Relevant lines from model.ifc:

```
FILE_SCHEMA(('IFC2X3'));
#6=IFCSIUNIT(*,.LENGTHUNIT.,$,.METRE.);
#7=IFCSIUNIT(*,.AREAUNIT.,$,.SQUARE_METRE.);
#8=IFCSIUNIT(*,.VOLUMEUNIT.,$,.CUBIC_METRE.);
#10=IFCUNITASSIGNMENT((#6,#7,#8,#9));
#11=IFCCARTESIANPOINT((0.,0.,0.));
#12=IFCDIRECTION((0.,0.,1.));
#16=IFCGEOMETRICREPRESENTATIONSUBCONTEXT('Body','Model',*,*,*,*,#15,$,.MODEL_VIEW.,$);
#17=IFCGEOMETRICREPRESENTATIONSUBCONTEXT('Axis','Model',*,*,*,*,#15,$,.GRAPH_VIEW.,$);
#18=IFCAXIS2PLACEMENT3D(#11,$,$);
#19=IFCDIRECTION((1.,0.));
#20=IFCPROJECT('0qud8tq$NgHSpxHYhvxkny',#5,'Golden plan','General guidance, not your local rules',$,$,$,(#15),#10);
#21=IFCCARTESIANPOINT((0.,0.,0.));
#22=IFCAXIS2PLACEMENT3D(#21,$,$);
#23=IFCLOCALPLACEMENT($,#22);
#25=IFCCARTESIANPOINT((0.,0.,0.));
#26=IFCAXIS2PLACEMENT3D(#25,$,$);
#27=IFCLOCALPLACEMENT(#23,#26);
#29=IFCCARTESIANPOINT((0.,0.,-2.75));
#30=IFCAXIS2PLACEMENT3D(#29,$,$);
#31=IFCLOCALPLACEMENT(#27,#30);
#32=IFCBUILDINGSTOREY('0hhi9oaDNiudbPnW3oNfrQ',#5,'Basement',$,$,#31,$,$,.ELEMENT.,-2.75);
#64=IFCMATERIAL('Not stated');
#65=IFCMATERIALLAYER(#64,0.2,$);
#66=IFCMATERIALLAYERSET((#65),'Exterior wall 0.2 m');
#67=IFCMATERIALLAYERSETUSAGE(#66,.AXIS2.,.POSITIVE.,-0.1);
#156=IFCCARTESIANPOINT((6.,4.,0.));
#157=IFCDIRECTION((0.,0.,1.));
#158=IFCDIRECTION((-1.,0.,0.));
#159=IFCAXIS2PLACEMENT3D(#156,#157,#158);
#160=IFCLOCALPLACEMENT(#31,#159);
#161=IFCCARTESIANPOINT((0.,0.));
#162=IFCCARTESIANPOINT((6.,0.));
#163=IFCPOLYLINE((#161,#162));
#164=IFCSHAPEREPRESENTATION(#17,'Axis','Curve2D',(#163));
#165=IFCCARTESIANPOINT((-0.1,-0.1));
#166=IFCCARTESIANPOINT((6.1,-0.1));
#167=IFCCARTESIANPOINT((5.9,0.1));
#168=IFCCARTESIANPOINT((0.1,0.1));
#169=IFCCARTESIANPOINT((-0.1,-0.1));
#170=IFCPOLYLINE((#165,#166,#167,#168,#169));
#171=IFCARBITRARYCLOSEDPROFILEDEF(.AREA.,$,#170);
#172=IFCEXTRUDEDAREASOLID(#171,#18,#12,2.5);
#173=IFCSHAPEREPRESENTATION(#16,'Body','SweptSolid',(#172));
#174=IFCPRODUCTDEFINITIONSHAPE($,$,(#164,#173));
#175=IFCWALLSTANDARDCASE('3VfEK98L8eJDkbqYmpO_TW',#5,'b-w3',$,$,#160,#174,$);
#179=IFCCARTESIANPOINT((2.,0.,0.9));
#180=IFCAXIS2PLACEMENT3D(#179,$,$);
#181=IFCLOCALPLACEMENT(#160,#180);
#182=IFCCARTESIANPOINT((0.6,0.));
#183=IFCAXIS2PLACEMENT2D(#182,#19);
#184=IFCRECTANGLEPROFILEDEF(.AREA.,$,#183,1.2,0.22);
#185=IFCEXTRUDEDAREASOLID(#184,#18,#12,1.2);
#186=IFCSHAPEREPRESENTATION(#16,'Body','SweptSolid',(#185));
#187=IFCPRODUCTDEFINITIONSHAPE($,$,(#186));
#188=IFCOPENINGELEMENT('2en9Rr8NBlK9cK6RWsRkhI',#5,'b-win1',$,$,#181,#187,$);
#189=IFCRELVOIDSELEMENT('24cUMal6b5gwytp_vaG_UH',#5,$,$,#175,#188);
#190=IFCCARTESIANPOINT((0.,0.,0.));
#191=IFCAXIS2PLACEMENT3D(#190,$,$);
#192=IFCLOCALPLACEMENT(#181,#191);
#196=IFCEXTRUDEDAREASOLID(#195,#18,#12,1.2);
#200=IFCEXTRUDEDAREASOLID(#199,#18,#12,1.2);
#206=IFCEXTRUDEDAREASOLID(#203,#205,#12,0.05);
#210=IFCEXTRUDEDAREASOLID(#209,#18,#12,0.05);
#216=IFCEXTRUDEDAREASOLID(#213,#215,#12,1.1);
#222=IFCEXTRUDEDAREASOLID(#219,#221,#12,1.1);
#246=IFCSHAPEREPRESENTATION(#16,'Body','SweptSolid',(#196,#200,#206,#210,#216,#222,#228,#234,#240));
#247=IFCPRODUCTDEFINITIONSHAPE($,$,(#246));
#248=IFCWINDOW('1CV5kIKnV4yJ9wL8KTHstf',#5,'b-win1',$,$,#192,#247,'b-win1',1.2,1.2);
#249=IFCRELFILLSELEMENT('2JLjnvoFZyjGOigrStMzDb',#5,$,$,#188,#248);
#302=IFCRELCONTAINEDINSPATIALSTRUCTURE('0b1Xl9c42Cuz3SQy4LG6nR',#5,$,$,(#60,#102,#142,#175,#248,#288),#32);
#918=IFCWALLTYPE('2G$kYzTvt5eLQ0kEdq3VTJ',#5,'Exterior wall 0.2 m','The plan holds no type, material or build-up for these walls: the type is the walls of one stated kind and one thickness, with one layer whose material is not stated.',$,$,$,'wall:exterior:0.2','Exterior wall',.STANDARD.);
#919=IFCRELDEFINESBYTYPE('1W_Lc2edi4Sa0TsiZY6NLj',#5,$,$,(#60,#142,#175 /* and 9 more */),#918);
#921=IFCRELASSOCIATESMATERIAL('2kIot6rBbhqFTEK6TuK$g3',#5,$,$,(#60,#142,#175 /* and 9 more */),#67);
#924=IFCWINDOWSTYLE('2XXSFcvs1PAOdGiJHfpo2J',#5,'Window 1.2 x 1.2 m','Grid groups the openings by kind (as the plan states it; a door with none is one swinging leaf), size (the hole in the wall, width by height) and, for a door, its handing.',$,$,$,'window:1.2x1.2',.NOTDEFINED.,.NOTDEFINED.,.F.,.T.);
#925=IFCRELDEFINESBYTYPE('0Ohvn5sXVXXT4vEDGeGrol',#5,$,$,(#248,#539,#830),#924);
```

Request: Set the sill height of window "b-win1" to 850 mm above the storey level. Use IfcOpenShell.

```python
import numpy as np
import ifcopenshell
import ifcopenshell.api.geometry
import ifcopenshell.geom
import ifcopenshell.util.element
import ifcopenshell.util.placement
import ifcopenshell.util.shape
import ifcopenshell.util.unit

model = ifcopenshell.open("model.ifc")
unit_scale = ifcopenshell.util.unit.calculate_unit_scale(model)

window = model.by_id(248)
opening = window.FillsVoids[0].RelatingOpeningElement
storey = ifcopenshell.util.element.get_container(window, ifc_class="IfcBuildingStorey")
level = ifcopenshell.util.placement.get_local_placement(storey.ObjectPlacement)[2, 3]

# The opening's origin need not be at the sill, so measure its lowest point.
shape = ifcopenshell.geom.create_shape(ifcopenshell.geom.settings(), opening)
bottom = ifcopenshell.util.shape.get_shape_bottom_elevation(shape, shape.geometry) / unit_scale
dz = level + 0.85 - bottom

shift = np.array([0.0, 0.0, dz])
# The window is placed relative to its opening, so it follows when the opening moves.
matrix = ifcopenshell.util.placement.get_local_placement(opening.ObjectPlacement)
matrix[:3, 3] += shift
ifcopenshell.api.geometry.edit_object_placement(
    model, product=opening, matrix=matrix, is_si=False, should_transform_children=True
)

print(f"moved by {dz * unit_scale:+.3f} m")

model.write("model_v2.ifc")
```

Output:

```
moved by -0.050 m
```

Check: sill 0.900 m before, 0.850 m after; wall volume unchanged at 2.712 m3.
